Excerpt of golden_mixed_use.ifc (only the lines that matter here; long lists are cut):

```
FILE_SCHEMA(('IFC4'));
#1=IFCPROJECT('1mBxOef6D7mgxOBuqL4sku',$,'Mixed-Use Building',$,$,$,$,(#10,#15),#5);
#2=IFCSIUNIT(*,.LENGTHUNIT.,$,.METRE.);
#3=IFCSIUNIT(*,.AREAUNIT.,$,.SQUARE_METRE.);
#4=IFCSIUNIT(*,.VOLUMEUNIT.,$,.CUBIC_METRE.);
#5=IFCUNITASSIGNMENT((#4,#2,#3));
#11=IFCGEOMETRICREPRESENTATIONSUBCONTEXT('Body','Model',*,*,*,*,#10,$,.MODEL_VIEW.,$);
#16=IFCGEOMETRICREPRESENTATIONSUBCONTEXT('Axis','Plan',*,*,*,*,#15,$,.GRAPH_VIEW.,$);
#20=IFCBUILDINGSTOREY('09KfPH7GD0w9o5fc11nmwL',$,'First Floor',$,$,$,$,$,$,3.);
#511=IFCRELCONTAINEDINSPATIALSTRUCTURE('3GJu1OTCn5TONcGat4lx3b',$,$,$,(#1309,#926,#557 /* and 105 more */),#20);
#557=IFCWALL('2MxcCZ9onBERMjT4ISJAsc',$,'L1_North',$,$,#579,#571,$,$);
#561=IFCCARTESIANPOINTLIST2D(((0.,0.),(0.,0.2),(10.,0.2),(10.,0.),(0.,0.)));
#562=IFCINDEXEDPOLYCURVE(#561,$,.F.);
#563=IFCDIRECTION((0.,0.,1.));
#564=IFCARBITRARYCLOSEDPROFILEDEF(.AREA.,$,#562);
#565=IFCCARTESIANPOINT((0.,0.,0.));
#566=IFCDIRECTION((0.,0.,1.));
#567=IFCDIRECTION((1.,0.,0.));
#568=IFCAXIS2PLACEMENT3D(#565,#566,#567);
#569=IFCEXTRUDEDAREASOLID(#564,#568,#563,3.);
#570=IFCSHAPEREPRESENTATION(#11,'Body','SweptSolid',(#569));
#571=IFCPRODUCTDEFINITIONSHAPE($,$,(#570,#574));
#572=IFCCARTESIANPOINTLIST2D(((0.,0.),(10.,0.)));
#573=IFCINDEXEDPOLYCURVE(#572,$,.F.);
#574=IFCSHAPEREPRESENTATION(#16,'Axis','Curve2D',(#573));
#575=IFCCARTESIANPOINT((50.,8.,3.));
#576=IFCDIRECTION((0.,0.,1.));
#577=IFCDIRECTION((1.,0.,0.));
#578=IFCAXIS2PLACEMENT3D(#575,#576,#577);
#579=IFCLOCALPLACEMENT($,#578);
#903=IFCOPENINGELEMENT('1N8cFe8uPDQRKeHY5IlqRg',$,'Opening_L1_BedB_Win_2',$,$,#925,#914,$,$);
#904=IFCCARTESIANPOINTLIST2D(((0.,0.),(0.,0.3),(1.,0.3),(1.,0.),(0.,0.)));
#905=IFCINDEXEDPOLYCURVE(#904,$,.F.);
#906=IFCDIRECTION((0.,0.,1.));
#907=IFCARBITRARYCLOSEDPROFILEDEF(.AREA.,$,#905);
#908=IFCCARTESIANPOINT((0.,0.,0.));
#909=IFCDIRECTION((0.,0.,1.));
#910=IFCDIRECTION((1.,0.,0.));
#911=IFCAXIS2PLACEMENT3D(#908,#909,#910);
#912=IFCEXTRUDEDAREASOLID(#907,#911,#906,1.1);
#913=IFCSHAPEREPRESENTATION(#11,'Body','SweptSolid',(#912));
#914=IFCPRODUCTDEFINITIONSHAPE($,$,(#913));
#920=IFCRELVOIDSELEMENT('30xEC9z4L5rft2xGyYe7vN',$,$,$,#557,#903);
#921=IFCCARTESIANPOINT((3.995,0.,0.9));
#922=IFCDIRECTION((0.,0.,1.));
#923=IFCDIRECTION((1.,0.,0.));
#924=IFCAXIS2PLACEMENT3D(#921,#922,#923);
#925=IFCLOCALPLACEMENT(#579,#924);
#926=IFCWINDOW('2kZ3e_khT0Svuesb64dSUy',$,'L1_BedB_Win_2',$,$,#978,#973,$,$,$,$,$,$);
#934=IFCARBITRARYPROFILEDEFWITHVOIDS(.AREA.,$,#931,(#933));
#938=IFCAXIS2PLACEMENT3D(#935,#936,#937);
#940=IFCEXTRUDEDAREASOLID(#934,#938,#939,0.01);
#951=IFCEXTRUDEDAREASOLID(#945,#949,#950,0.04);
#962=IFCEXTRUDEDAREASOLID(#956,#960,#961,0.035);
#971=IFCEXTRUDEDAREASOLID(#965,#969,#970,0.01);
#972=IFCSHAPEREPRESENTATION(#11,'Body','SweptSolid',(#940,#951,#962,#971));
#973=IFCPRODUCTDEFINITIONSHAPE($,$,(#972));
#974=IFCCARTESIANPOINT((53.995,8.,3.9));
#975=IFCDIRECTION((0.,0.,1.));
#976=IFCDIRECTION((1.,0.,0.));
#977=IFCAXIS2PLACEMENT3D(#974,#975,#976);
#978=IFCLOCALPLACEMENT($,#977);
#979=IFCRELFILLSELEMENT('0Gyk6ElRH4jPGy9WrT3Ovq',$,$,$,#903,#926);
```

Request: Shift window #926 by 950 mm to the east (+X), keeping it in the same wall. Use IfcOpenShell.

```python
import ifcopenshell
import ifcopenshell.api.geometry
import ifcopenshell.util.placement

model = ifcopenshell.open("golden_mixed_use.ifc")

window = model.by_id(926)
opening = window.FillsVoids[0].RelatingOpeningElement
wall = opening.VoidsElements[0].RelatingBuildingElement

wall_matrix = ifcopenshell.util.placement.get_local_placement(wall.ObjectPlacement)
shift = wall_matrix[:3, 0] * 0.95
before = ifcopenshell.util.placement.get_local_placement(window.ObjectPlacement)[:3, 3].copy()

# The window is not placed relative to its opening, so move both.
for product in (opening, window):
    matrix = ifcopenshell.util.placement.get_local_placement(product.ObjectPlacement)
    matrix[:3, 3] += shift
    ifcopenshell.api.geometry.edit_object_placement(model, product=product, matrix=matrix, is_si=False)

after = ifcopenshell.util.placement.get_local_placement(window.ObjectPlacement)[:3, 3]
print("window moved by", (after - before).round(3) + 0.0)

model.write("golden_mixed_use_rev.ifc")
```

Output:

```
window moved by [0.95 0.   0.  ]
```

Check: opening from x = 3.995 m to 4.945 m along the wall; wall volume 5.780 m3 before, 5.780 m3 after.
